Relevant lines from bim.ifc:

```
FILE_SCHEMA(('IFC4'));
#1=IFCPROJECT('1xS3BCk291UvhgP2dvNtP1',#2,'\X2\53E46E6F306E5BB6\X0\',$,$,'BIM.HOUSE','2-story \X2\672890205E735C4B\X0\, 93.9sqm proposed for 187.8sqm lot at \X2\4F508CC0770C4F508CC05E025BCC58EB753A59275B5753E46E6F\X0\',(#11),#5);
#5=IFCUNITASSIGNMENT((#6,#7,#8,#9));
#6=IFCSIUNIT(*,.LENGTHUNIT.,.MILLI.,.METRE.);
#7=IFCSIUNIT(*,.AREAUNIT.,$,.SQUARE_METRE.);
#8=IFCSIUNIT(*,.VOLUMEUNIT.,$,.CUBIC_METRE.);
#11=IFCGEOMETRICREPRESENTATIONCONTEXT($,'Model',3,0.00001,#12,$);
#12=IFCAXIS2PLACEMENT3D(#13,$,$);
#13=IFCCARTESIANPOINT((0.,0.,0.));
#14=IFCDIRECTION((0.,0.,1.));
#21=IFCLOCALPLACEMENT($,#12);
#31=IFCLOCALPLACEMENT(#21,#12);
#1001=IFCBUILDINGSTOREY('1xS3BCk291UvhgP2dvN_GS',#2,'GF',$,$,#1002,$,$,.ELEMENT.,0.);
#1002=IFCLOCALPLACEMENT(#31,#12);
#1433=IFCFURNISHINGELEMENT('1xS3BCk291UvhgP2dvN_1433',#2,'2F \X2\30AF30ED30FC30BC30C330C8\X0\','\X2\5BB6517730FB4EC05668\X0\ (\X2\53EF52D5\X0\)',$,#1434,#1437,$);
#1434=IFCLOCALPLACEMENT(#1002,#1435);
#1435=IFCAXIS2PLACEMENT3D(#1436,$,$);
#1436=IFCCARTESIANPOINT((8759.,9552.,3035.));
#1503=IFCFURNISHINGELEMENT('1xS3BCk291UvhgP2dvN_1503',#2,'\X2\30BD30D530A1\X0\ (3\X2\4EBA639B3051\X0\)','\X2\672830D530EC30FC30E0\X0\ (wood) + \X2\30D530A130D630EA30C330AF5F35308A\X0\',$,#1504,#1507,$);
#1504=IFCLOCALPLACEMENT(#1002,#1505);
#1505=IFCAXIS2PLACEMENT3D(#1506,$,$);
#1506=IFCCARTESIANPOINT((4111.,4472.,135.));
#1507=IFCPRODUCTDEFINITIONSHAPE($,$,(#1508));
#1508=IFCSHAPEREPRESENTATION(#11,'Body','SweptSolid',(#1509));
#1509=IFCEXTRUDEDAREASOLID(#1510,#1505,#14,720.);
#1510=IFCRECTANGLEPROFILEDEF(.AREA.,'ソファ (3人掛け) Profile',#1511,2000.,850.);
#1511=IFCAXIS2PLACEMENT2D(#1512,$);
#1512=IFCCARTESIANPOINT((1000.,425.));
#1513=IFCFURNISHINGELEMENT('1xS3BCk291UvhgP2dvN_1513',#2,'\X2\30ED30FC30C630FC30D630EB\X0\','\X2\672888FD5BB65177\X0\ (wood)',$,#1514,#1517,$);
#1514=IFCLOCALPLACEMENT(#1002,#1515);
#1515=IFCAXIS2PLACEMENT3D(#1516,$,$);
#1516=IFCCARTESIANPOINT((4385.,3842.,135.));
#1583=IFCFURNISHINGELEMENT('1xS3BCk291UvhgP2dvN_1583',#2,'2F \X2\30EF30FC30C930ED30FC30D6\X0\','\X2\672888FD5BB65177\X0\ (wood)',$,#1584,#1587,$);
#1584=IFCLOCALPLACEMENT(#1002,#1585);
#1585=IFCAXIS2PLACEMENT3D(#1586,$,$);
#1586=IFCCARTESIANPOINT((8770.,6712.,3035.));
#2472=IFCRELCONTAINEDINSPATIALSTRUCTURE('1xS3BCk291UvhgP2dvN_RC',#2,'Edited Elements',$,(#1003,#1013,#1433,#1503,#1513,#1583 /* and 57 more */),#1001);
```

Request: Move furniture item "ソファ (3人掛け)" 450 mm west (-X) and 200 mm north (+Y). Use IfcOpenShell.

```python
import ifcopenshell
import ifcopenshell.api.geometry
import ifcopenshell.util.placement
import ifcopenshell.util.unit

model = ifcopenshell.open("bim.ifc")
unit_scale = ifcopenshell.util.unit.calculate_unit_scale(model)

item = model.by_guid("1xS3BCk291UvhgP2dvN_1503")
matrix = ifcopenshell.util.placement.get_local_placement(item.ObjectPlacement)
matrix[0, 3] -= 0.45 / unit_scale
matrix[1, 3] += 0.2 / unit_scale
ifcopenshell.api.geometry.edit_object_placement(model, product=item, matrix=matrix, is_si=False)

print(ifcopenshell.util.placement.get_local_placement(item.ObjectPlacement).round(3) + 0.0)

model.write("bim_edited.ifc")
```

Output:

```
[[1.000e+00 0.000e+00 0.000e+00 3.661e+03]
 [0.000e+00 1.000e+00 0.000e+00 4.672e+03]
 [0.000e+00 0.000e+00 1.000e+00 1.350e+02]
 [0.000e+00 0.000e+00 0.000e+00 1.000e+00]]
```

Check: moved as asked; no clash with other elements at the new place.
